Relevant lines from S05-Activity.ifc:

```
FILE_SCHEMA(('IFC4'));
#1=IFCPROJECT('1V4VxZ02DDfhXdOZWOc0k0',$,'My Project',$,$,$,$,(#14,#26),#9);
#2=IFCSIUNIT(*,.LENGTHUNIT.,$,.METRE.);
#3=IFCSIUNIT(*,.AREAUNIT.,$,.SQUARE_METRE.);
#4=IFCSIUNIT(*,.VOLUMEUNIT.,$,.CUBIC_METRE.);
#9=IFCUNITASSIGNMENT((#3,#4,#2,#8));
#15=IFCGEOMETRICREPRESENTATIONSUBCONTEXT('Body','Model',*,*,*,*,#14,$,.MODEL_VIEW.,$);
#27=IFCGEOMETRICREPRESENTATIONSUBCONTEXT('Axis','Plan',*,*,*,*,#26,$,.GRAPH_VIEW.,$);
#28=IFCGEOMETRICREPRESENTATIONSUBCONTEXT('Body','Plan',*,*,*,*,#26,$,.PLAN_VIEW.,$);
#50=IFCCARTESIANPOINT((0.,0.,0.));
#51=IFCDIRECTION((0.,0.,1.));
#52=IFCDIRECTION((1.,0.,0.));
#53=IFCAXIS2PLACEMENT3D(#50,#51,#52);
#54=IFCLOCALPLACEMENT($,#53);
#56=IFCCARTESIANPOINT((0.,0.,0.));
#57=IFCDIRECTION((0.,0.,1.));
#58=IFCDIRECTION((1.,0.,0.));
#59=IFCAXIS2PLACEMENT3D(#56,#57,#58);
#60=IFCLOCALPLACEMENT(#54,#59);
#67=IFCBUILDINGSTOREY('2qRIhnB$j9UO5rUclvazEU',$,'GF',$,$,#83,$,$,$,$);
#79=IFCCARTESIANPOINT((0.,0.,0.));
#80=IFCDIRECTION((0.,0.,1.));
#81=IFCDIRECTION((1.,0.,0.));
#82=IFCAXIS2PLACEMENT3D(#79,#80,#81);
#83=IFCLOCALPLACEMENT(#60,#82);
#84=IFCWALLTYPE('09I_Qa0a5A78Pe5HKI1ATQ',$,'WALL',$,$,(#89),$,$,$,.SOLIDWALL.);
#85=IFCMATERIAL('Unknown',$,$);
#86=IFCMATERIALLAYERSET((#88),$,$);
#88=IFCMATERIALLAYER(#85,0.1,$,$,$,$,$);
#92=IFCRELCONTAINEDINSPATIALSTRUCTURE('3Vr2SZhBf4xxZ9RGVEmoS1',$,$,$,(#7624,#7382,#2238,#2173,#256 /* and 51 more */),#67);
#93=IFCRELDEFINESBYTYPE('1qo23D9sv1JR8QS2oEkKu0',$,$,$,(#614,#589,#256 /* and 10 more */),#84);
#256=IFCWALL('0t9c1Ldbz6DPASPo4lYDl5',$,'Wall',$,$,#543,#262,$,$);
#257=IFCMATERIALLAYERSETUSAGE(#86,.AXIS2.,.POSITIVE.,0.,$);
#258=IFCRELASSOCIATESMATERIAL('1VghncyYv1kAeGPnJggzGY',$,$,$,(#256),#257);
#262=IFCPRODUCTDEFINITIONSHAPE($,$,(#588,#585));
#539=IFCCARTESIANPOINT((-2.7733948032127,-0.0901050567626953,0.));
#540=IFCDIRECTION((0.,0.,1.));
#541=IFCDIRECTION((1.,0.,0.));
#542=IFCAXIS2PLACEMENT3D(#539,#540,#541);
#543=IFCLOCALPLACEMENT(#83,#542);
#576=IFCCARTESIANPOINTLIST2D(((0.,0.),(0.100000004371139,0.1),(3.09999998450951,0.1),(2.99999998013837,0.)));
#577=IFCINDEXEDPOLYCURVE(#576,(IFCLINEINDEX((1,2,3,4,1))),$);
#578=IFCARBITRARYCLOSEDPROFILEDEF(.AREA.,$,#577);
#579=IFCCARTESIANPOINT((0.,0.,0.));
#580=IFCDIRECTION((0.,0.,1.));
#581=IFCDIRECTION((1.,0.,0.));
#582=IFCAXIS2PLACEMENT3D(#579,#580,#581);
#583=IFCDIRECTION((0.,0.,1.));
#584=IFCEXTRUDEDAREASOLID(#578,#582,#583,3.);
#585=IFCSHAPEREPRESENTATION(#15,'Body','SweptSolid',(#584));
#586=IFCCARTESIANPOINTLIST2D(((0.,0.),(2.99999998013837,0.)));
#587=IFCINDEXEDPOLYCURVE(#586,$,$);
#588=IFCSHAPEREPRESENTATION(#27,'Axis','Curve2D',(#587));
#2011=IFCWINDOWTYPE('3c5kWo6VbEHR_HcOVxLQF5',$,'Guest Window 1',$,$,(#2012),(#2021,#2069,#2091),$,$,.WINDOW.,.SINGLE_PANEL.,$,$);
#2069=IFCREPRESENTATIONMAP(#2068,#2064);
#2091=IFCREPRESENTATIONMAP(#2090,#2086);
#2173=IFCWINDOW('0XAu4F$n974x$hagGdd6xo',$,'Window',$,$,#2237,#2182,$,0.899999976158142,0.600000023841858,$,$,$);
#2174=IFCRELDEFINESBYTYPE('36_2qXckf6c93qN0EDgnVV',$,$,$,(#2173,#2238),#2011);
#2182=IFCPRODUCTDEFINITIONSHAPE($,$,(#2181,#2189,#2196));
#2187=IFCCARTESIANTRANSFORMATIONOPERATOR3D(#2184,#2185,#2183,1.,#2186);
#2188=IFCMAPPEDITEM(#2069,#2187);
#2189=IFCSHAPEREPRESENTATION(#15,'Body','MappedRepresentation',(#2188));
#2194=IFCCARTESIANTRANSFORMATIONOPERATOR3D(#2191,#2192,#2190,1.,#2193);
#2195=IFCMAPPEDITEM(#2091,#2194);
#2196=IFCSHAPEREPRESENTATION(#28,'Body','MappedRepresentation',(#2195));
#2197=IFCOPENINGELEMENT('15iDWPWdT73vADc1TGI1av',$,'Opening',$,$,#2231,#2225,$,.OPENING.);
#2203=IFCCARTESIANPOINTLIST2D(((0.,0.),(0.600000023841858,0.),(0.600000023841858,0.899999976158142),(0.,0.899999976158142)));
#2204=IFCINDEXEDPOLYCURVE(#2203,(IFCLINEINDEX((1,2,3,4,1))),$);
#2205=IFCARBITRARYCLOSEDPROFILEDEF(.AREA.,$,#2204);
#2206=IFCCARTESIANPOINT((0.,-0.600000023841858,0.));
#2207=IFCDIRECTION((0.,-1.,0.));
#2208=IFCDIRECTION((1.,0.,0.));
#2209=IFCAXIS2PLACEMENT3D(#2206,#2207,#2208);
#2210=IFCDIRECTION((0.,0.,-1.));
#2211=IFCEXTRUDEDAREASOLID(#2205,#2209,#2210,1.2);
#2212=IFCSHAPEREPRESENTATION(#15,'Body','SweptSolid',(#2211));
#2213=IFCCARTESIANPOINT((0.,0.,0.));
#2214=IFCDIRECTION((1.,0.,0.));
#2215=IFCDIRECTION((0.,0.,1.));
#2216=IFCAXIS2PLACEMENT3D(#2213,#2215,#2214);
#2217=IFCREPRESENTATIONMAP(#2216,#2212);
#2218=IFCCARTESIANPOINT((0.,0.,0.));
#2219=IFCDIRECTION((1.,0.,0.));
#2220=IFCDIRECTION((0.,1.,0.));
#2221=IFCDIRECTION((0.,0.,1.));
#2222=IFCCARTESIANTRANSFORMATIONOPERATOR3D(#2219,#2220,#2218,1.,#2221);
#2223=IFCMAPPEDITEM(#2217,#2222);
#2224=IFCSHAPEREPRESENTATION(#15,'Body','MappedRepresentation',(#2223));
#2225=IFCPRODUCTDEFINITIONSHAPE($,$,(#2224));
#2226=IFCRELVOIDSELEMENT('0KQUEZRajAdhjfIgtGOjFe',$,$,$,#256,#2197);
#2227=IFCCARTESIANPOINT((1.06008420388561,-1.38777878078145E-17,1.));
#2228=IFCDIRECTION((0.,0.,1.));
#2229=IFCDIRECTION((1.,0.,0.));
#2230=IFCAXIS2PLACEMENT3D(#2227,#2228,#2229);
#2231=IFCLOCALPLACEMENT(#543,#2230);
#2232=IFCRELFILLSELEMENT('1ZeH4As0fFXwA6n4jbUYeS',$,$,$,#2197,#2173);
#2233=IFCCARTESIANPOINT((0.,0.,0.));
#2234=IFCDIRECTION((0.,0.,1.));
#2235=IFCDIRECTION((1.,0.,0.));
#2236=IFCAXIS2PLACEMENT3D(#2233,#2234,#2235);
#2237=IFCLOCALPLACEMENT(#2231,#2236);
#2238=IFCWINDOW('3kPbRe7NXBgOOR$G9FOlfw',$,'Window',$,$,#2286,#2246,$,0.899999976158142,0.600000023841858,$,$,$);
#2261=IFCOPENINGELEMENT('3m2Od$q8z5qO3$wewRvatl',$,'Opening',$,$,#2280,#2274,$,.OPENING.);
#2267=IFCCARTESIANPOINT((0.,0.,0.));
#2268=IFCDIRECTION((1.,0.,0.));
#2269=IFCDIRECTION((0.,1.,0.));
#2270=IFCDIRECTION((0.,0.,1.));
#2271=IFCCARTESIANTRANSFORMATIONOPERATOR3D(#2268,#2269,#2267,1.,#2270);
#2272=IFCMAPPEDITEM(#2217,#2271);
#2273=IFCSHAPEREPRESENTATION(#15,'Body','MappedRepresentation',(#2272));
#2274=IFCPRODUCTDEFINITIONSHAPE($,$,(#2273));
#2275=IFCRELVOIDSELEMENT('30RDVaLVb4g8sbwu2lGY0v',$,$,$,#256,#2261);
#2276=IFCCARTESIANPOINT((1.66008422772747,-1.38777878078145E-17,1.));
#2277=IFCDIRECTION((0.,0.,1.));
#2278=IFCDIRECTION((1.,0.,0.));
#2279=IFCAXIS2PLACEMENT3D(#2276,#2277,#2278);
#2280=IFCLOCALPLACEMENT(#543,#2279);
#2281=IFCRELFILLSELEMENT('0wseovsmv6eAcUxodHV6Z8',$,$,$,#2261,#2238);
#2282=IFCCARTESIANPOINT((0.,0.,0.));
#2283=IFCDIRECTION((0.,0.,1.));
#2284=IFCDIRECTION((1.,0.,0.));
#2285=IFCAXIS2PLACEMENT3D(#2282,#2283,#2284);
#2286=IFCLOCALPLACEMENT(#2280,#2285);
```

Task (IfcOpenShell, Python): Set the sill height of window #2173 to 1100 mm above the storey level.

```python
import numpy as np
import ifcopenshell
import ifcopenshell.api.geometry
import ifcopenshell.geom
import ifcopenshell.util.element
import ifcopenshell.util.placement
import ifcopenshell.util.shape
import ifcopenshell.util.unit

model = ifcopenshell.open("S05-Activity.ifc")
unit_scale = ifcopenshell.util.unit.calculate_unit_scale(model)

window = model.by_guid("0XAu4F$n974x$hagGdd6xo")
opening = window.FillsVoids[0].RelatingOpeningElement
storey = ifcopenshell.util.element.get_container(window, ifc_class="IfcBuildingStorey")
level = ifcopenshell.util.placement.get_local_placement(storey.ObjectPlacement)[2, 3]

# The opening's origin need not be at the sill, so measure its lowest point.
shape = ifcopenshell.geom.create_shape(ifcopenshell.geom.settings(), opening)
bottom = ifcopenshell.util.shape.get_shape_bottom_elevation(shape, shape.geometry) / unit_scale
dz = level + 1.1 / unit_scale - bottom

shift = np.array([0.0, 0.0, dz])
# The window is placed relative to its opening, so it follows when the opening moves.
matrix = ifcopenshell.util.placement.get_local_placement(opening.ObjectPlacement)
matrix[:3, 3] += shift
ifcopenshell.api.geometry.edit_object_placement(
    model, product=opening, matrix=matrix, is_si=False, should_transform_children=True
)

print(f"moved by {dz * unit_scale:+.3f} m")

model.write("S05-Activity_v2.ifc")
```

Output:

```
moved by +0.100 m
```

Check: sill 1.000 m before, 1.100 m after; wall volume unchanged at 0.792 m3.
